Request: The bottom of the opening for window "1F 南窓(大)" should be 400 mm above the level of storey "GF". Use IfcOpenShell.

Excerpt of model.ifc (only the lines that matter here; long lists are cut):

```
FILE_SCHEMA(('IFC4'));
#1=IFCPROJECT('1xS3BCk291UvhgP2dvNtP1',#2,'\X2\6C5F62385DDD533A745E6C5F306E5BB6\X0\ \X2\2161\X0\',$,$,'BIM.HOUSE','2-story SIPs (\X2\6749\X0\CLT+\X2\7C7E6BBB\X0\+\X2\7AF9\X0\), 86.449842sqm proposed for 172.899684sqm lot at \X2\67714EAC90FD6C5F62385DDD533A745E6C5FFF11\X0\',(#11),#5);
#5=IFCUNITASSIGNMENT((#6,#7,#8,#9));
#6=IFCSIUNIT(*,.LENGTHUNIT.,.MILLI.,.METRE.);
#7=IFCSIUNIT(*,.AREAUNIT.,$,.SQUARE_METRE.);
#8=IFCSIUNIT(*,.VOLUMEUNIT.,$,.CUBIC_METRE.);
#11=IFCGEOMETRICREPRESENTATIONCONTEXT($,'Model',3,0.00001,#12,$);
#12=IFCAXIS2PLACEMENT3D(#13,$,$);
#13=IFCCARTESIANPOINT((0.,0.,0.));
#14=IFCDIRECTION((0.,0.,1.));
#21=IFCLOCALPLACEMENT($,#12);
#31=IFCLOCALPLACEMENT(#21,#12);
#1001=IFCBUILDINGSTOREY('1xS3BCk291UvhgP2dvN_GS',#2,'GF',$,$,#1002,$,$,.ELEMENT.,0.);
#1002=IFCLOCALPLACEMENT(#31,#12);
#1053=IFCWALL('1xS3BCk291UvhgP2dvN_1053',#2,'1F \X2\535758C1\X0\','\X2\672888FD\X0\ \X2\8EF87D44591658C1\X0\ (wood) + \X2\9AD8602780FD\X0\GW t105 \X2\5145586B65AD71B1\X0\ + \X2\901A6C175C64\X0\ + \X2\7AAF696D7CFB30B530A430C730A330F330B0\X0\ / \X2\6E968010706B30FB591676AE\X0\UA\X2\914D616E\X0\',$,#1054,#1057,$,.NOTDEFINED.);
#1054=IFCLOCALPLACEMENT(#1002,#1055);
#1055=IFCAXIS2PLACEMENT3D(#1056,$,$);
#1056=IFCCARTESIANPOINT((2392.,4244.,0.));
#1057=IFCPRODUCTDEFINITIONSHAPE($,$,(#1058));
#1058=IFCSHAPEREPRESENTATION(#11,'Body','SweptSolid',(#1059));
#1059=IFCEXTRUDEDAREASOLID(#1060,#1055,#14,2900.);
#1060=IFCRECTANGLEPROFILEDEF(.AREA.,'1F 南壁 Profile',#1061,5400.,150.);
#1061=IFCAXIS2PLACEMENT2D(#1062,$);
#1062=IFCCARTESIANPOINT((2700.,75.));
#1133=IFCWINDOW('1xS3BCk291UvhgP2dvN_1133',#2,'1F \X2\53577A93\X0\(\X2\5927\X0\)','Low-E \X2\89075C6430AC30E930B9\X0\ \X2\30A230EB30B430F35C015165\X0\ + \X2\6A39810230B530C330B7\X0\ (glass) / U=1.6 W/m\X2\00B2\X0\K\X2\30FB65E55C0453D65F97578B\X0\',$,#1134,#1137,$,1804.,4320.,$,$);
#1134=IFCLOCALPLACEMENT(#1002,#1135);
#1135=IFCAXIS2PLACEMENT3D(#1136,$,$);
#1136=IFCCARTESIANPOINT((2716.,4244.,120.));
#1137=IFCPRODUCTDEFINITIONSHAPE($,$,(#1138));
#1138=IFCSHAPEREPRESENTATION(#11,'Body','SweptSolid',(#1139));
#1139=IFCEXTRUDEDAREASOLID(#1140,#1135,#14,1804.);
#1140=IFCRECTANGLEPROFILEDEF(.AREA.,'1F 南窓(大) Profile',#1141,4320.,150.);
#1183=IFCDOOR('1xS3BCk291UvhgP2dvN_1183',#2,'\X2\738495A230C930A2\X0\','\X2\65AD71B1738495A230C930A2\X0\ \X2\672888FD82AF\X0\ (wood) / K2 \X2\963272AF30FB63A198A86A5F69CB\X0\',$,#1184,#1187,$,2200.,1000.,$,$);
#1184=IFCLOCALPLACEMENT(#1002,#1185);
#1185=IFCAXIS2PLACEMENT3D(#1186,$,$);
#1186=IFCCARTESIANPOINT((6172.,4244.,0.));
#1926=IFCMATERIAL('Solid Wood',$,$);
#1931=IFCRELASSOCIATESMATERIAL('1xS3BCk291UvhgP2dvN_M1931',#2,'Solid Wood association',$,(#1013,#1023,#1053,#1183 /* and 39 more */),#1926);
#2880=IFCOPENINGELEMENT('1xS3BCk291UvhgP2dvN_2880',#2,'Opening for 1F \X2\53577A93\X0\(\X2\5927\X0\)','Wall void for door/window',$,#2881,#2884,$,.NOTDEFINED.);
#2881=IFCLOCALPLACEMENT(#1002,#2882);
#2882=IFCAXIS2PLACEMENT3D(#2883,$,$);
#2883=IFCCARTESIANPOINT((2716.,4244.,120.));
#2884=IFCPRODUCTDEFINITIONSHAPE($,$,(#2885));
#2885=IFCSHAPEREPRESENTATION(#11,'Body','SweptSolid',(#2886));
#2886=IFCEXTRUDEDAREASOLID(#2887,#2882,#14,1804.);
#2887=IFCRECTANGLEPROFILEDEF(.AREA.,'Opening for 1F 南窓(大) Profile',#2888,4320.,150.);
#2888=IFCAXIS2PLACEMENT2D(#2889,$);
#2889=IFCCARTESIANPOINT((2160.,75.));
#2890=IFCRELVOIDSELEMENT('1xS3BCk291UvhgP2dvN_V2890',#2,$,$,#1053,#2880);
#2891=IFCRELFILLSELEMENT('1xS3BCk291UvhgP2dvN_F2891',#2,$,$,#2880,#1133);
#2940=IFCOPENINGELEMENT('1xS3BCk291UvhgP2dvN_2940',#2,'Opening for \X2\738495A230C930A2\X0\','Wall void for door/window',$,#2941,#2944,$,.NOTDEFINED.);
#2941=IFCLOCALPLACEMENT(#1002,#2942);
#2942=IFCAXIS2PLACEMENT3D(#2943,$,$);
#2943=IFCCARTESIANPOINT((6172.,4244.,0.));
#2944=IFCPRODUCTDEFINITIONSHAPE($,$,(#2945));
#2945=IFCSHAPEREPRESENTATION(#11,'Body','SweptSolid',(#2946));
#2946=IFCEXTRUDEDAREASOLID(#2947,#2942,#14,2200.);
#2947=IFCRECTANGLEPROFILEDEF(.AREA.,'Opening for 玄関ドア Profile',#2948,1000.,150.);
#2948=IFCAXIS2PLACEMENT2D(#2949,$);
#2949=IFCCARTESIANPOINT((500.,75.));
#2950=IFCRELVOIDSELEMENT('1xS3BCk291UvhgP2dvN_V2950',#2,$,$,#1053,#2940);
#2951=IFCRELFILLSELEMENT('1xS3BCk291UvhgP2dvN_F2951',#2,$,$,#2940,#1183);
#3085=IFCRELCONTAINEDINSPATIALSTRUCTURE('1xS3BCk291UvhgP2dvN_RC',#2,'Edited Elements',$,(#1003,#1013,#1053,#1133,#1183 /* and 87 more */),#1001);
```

```python
import numpy as np
import ifcopenshell
import ifcopenshell.api.geometry
import ifcopenshell.geom
import ifcopenshell.util.element
import ifcopenshell.util.placement
import ifcopenshell.util.shape
import ifcopenshell.util.unit

model = ifcopenshell.open("model.ifc")
unit_scale = ifcopenshell.util.unit.calculate_unit_scale(model)

window = model.by_guid("1xS3BCk291UvhgP2dvN_1133")
opening = window.FillsVoids[0].RelatingOpeningElement
storey = ifcopenshell.util.element.get_container(window, ifc_class="IfcBuildingStorey")
level = ifcopenshell.util.placement.get_local_placement(storey.ObjectPlacement)[2, 3]

# The opening's origin need not be at the sill, so measure its lowest point.
shape = ifcopenshell.geom.create_shape(ifcopenshell.geom.settings(), opening)
bottom = ifcopenshell.util.shape.get_shape_bottom_elevation(shape, shape.geometry) / unit_scale
dz = level + 400.0 - bottom

shift = np.array([0.0, 0.0, dz])
# The window is not placed relative to its opening, so move both.
for product in (opening, window):
    matrix = ifcopenshell.util.placement.get_local_placement(product.ObjectPlacement)
    matrix[:3, 3] += shift
    ifcopenshell.api.geometry.edit_object_placement(model, product=product, matrix=matrix, is_si=False)

print(f"moved by {dz * unit_scale:+.3f} m")

model.write("model_v2.ifc")
```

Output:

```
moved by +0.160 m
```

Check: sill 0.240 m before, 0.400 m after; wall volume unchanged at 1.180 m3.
